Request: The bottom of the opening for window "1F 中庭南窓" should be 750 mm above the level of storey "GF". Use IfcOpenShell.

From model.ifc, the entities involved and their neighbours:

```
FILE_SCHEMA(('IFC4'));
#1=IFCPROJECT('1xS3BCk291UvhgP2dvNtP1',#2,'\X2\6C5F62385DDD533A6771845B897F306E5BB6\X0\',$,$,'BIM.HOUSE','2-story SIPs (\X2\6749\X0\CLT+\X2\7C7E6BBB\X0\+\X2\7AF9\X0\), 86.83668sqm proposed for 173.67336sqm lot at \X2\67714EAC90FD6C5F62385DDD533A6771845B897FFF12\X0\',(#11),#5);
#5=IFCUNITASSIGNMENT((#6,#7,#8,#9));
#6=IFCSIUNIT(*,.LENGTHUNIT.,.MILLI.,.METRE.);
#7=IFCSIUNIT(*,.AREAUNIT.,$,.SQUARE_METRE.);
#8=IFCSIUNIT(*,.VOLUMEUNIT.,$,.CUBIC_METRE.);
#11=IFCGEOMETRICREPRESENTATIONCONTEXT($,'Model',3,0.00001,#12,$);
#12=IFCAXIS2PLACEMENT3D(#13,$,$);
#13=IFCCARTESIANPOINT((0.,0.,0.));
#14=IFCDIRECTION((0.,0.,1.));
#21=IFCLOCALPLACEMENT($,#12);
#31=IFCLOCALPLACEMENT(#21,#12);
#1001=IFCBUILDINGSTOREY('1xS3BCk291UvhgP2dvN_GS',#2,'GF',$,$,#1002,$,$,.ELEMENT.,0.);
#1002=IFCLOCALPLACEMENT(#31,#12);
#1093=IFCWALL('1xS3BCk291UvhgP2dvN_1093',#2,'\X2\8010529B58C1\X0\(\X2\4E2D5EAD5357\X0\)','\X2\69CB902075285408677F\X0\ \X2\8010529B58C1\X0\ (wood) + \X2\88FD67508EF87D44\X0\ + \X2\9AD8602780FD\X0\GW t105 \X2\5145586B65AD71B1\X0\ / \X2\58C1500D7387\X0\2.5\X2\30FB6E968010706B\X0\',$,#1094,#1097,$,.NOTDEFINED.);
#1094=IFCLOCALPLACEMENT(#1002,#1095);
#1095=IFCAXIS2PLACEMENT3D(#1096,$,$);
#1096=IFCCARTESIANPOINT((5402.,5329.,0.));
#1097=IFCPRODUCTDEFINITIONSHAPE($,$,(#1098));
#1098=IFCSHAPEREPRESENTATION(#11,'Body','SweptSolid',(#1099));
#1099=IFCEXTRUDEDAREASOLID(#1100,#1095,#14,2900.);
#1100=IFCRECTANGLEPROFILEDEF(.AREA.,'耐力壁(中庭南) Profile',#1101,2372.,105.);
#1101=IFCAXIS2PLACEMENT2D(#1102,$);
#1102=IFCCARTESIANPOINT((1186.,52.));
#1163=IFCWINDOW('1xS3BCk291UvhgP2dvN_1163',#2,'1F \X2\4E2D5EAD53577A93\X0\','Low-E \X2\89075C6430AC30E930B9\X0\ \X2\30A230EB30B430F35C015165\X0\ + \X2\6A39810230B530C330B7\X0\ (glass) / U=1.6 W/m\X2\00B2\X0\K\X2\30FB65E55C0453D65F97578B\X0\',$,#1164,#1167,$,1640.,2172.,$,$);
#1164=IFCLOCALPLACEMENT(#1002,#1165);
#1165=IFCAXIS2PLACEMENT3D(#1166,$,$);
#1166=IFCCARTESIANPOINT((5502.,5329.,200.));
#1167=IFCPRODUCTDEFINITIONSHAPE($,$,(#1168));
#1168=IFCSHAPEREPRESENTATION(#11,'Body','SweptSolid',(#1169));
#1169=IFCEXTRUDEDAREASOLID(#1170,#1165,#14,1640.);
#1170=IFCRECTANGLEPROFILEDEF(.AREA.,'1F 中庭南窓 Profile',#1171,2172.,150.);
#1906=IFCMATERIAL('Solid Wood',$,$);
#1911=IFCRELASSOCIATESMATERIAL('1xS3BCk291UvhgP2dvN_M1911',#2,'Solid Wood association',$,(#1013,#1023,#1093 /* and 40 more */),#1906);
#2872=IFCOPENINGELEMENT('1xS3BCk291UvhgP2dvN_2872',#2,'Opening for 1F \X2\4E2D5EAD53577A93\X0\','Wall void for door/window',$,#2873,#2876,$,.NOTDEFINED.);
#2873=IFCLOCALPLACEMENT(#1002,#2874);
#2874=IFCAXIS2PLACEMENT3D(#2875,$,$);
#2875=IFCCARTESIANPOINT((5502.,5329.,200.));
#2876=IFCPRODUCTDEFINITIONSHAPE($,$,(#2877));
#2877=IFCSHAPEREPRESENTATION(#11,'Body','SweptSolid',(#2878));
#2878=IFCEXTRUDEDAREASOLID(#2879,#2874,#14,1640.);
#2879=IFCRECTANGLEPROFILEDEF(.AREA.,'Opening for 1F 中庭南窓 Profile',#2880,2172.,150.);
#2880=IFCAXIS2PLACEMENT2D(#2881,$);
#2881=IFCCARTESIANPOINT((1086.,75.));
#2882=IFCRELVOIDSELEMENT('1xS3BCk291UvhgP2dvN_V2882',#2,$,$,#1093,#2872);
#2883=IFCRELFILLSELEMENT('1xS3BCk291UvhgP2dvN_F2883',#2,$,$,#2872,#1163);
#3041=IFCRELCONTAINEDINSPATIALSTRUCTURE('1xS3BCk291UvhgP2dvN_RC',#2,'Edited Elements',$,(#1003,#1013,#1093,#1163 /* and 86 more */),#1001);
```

```python
import numpy as np
import ifcopenshell
import ifcopenshell.api.geometry
import ifcopenshell.geom
import ifcopenshell.util.element
import ifcopenshell.util.placement
import ifcopenshell.util.shape
import ifcopenshell.util.unit

model = ifcopenshell.open("model.ifc")
unit_scale = ifcopenshell.util.unit.calculate_unit_scale(model)

window = model.by_guid("1xS3BCk291UvhgP2dvN_1163")
opening = window.FillsVoids[0].RelatingOpeningElement
storey = ifcopenshell.util.element.get_container(window, ifc_class="IfcBuildingStorey")
level = ifcopenshell.util.placement.get_local_placement(storey.ObjectPlacement)[2, 3]

# The opening's origin need not be at the sill, so measure its lowest point.
shape = ifcopenshell.geom.create_shape(ifcopenshell.geom.settings(), opening)
bottom = ifcopenshell.util.shape.get_shape_bottom_elevation(shape, shape.geometry) / unit_scale
dz = level + 0.75 / unit_scale - bottom

shift = np.array([0.0, 0.0, dz])
# The window is not placed relative to its opening, so move both.
for product in (opening, window):
    matrix = ifcopenshell.util.placement.get_local_placement(product.ObjectPlacement)
    matrix[:3, 3] += shift
    ifcopenshell.api.geometry.edit_object_placement(model, product=product, matrix=matrix, is_si=False)

print(f"moved by {dz * unit_scale:+.3f} m")

model.write("model_edited.ifc")
```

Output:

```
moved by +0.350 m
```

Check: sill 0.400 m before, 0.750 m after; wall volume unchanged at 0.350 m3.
